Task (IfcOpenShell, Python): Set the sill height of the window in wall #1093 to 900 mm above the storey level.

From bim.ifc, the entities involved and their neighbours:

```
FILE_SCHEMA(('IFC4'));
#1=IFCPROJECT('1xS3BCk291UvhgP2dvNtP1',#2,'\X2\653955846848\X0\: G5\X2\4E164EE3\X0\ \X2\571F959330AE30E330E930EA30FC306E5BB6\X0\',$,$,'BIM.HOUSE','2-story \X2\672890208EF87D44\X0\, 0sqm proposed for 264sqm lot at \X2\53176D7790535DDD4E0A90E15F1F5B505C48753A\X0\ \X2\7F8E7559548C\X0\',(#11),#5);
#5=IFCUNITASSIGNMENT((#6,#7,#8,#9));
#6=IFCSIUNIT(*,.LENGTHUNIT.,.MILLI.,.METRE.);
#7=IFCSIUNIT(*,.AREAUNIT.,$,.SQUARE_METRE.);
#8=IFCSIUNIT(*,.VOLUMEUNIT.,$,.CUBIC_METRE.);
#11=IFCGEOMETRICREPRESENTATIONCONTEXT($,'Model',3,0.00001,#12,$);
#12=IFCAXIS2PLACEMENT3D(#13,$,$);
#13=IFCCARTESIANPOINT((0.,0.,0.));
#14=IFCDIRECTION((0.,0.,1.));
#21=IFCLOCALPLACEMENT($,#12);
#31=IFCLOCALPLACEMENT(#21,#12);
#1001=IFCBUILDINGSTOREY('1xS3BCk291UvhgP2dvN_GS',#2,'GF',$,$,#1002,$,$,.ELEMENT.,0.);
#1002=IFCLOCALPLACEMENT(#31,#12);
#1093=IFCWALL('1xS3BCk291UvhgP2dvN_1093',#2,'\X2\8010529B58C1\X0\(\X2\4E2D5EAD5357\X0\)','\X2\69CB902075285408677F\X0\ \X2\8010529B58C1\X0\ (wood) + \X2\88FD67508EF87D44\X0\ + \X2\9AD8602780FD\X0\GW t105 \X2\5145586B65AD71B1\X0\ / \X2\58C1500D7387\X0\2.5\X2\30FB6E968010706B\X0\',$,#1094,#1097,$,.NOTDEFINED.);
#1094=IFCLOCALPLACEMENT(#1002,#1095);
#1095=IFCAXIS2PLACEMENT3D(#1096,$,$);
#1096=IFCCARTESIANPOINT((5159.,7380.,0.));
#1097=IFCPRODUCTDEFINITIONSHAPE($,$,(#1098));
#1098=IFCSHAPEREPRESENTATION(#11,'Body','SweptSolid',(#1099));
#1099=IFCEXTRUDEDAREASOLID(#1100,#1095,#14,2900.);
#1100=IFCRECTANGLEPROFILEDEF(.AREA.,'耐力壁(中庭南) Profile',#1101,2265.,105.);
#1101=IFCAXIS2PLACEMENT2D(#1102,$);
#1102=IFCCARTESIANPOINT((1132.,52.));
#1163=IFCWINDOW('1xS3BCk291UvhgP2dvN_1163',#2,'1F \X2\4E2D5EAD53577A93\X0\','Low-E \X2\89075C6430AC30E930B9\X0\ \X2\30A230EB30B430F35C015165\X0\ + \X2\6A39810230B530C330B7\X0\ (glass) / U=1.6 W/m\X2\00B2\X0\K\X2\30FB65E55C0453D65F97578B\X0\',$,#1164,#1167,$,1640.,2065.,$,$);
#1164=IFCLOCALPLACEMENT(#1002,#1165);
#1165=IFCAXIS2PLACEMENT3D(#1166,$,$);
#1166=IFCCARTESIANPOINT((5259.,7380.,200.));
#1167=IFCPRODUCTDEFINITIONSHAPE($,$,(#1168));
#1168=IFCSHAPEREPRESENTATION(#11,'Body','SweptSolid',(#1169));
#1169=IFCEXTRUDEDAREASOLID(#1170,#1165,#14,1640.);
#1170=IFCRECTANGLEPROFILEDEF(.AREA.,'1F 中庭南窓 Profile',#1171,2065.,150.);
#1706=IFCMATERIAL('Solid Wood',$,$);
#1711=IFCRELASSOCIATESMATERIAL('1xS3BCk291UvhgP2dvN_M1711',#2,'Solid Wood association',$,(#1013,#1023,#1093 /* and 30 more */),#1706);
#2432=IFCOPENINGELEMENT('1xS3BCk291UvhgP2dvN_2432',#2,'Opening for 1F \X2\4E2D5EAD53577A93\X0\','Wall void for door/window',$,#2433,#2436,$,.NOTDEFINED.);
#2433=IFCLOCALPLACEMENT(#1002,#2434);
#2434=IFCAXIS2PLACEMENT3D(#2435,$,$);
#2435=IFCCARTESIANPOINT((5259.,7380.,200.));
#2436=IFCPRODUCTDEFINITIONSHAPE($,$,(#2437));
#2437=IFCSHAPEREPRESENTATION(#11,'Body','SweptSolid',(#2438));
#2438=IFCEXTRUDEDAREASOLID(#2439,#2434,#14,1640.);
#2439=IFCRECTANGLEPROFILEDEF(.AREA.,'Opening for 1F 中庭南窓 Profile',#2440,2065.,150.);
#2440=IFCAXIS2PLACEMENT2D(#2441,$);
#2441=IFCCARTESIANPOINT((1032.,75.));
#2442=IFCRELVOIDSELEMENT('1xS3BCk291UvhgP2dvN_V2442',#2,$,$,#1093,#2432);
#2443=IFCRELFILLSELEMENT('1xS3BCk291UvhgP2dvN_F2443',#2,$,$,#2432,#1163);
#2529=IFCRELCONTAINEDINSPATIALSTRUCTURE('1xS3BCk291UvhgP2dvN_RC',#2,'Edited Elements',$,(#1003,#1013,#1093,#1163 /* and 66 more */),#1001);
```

```python
import numpy as np
import ifcopenshell
import ifcopenshell.api.geometry
import ifcopenshell.geom
import ifcopenshell.util.element
import ifcopenshell.util.placement
import ifcopenshell.util.shape
import ifcopenshell.util.unit

model = ifcopenshell.open("bim.ifc")
unit_scale = ifcopenshell.util.unit.calculate_unit_scale(model)

window = model.by_guid("1xS3BCk291UvhgP2dvN_1163")
opening = window.FillsVoids[0].RelatingOpeningElement
storey = ifcopenshell.util.element.get_container(window, ifc_class="IfcBuildingStorey")
level = ifcopenshell.util.placement.get_local_placement(storey.ObjectPlacement)[2, 3]

# The opening's origin need not be at the sill, so measure its lowest point.
shape = ifcopenshell.geom.create_shape(ifcopenshell.geom.settings(), opening)
bottom = ifcopenshell.util.shape.get_shape_bottom_elevation(shape, shape.geometry) / unit_scale
dz = level + 0.9 / unit_scale - bottom

shift = np.array([0.0, 0.0, dz])
# The window is not placed relative to its opening, so move both.
for product in (opening, window):
    matrix = ifcopenshell.util.placement.get_local_placement(product.ObjectPlacement)
    matrix[:3, 3] += shift
    ifcopenshell.api.geometry.edit_object_placement(model, product=product, matrix=matrix, is_si=False)

print(f"moved by {dz * unit_scale:+.3f} m")

model.write("bim_edited.ifc")
```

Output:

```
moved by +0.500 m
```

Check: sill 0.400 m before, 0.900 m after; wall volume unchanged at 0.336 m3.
